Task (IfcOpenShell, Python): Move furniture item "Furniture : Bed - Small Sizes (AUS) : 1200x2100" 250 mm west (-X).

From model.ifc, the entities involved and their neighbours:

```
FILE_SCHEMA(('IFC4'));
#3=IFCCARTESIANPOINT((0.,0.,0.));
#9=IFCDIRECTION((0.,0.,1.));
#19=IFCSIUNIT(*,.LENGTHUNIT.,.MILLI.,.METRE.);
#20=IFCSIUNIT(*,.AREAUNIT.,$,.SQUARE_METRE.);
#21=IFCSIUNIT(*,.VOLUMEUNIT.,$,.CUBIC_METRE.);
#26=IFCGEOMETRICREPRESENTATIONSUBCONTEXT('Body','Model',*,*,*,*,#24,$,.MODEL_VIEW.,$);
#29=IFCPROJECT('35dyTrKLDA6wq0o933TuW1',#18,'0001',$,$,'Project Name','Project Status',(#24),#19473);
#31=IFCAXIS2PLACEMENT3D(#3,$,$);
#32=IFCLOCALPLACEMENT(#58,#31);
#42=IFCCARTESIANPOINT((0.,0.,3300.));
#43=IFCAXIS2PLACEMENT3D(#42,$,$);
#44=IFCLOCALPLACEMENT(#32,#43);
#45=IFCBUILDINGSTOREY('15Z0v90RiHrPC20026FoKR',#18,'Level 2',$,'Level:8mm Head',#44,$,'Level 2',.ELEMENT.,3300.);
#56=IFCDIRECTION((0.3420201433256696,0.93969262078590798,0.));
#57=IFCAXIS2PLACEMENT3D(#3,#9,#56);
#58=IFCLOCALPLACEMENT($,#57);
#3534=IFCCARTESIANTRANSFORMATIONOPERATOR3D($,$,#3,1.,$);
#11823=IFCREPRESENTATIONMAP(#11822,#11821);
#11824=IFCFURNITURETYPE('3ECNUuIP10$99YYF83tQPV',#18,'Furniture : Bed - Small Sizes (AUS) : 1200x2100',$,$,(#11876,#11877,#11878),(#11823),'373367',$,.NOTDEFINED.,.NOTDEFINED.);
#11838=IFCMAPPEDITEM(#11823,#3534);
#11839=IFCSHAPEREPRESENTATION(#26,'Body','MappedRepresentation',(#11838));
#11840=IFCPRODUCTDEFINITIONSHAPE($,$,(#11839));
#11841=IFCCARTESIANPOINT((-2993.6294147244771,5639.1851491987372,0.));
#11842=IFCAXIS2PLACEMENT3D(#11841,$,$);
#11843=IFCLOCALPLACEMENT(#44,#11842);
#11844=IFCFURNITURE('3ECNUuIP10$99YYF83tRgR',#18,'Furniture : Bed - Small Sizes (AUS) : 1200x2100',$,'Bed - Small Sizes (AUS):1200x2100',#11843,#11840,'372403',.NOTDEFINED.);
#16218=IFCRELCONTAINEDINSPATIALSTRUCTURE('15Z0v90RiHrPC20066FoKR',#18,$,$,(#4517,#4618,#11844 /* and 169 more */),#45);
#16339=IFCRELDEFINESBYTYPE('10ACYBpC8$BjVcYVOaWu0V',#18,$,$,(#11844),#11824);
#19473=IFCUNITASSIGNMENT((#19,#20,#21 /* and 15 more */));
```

```python
import ifcopenshell
import ifcopenshell.api.geometry
import ifcopenshell.util.placement

model = ifcopenshell.open("model.ifc")

item = model.by_guid("3ECNUuIP10$99YYF83tRgR")
matrix = ifcopenshell.util.placement.get_local_placement(item.ObjectPlacement)
matrix[0, 3] -= 250.0
ifcopenshell.api.geometry.edit_object_placement(model, product=item, matrix=matrix, is_si=False)

print(ifcopenshell.util.placement.get_local_placement(item.ObjectPlacement).round(3) + 0.0)

model.write("model_rev.ifc")
```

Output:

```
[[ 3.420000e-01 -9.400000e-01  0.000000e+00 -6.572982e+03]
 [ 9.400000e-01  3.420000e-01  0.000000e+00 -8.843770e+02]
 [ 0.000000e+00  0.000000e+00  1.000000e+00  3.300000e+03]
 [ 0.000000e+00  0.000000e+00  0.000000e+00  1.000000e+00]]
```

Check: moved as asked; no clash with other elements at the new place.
